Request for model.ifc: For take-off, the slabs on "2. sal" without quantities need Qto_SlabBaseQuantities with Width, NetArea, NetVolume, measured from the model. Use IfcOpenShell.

First a look at what the model holds.

```python
import ifcopenshell
import ifcopenshell.util.element
import ifcopenshell.util.unit

model = ifcopenshell.open("model.ifc")
print(model.schema)
for unit_type in ("LENGTHUNIT", "AREAUNIT", "VOLUMEUNIT"):
    print(unit_type, ifcopenshell.util.unit.calculate_unit_scale(model, unit_type))
storey = next(s for s in model.by_type("IfcBuildingStorey") if s.Name == "2. sal")
slabs = [e for e in ifcopenshell.util.element.get_decomposition(storey) if e.is_a("IfcSlab")]
for e in sorted(slabs, key=lambda e: e.id()):
    print(e.id(), e.is_a(), e.Name, list(ifcopenshell.util.element.get_psets(e, qtos_only=True)), sep=" | ")
```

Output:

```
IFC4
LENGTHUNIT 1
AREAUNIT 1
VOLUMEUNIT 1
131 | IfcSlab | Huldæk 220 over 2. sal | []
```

```python
import ifcopenshell
import ifcopenshell.api.pset
import ifcopenshell.geom
import ifcopenshell.util.element
import ifcopenshell.util.shape
import ifcopenshell.util.unit

model = ifcopenshell.open("model.ifc")
unit_scale = ifcopenshell.util.unit.calculate_unit_scale(model)
area_scale = ifcopenshell.util.unit.calculate_unit_scale(model, "AREAUNIT")
volume_scale = ifcopenshell.util.unit.calculate_unit_scale(model, "VOLUMEUNIT")
settings = ifcopenshell.geom.settings()

storey = next(s for s in model.by_type("IfcBuildingStorey") if s.Name == "2. sal")
slabs = [e for e in ifcopenshell.util.element.get_decomposition(storey) if e.is_a("IfcSlab")]

for e in sorted(slabs, key=lambda e: e.id()):
    if ifcopenshell.util.element.get_psets(e, qtos_only=True, should_inherit=False):
        continue
    # Geometry comes back in metres, in the element's own axes.
    shape = ifcopenshell.geom.create_shape(settings, e)
    values = {
        "Width": ifcopenshell.util.shape.get_z(shape.geometry) / unit_scale,
        "NetArea": ifcopenshell.util.shape.get_footprint_area(shape.geometry) / area_scale,
        "NetVolume": ifcopenshell.util.shape.get_volume(shape.geometry) / volume_scale,
    }
    qto = ifcopenshell.api.pset.add_qto(model, product=e, name="Qto_SlabBaseQuantities")
    ifcopenshell.api.pset.edit_qto(model, qto=qto, properties=values)
    print(e.id(), {k: round(v, 3) for k, v in values.items()})

model.write("model_v2.ifc")
```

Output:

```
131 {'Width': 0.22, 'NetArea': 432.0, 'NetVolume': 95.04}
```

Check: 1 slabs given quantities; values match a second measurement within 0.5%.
